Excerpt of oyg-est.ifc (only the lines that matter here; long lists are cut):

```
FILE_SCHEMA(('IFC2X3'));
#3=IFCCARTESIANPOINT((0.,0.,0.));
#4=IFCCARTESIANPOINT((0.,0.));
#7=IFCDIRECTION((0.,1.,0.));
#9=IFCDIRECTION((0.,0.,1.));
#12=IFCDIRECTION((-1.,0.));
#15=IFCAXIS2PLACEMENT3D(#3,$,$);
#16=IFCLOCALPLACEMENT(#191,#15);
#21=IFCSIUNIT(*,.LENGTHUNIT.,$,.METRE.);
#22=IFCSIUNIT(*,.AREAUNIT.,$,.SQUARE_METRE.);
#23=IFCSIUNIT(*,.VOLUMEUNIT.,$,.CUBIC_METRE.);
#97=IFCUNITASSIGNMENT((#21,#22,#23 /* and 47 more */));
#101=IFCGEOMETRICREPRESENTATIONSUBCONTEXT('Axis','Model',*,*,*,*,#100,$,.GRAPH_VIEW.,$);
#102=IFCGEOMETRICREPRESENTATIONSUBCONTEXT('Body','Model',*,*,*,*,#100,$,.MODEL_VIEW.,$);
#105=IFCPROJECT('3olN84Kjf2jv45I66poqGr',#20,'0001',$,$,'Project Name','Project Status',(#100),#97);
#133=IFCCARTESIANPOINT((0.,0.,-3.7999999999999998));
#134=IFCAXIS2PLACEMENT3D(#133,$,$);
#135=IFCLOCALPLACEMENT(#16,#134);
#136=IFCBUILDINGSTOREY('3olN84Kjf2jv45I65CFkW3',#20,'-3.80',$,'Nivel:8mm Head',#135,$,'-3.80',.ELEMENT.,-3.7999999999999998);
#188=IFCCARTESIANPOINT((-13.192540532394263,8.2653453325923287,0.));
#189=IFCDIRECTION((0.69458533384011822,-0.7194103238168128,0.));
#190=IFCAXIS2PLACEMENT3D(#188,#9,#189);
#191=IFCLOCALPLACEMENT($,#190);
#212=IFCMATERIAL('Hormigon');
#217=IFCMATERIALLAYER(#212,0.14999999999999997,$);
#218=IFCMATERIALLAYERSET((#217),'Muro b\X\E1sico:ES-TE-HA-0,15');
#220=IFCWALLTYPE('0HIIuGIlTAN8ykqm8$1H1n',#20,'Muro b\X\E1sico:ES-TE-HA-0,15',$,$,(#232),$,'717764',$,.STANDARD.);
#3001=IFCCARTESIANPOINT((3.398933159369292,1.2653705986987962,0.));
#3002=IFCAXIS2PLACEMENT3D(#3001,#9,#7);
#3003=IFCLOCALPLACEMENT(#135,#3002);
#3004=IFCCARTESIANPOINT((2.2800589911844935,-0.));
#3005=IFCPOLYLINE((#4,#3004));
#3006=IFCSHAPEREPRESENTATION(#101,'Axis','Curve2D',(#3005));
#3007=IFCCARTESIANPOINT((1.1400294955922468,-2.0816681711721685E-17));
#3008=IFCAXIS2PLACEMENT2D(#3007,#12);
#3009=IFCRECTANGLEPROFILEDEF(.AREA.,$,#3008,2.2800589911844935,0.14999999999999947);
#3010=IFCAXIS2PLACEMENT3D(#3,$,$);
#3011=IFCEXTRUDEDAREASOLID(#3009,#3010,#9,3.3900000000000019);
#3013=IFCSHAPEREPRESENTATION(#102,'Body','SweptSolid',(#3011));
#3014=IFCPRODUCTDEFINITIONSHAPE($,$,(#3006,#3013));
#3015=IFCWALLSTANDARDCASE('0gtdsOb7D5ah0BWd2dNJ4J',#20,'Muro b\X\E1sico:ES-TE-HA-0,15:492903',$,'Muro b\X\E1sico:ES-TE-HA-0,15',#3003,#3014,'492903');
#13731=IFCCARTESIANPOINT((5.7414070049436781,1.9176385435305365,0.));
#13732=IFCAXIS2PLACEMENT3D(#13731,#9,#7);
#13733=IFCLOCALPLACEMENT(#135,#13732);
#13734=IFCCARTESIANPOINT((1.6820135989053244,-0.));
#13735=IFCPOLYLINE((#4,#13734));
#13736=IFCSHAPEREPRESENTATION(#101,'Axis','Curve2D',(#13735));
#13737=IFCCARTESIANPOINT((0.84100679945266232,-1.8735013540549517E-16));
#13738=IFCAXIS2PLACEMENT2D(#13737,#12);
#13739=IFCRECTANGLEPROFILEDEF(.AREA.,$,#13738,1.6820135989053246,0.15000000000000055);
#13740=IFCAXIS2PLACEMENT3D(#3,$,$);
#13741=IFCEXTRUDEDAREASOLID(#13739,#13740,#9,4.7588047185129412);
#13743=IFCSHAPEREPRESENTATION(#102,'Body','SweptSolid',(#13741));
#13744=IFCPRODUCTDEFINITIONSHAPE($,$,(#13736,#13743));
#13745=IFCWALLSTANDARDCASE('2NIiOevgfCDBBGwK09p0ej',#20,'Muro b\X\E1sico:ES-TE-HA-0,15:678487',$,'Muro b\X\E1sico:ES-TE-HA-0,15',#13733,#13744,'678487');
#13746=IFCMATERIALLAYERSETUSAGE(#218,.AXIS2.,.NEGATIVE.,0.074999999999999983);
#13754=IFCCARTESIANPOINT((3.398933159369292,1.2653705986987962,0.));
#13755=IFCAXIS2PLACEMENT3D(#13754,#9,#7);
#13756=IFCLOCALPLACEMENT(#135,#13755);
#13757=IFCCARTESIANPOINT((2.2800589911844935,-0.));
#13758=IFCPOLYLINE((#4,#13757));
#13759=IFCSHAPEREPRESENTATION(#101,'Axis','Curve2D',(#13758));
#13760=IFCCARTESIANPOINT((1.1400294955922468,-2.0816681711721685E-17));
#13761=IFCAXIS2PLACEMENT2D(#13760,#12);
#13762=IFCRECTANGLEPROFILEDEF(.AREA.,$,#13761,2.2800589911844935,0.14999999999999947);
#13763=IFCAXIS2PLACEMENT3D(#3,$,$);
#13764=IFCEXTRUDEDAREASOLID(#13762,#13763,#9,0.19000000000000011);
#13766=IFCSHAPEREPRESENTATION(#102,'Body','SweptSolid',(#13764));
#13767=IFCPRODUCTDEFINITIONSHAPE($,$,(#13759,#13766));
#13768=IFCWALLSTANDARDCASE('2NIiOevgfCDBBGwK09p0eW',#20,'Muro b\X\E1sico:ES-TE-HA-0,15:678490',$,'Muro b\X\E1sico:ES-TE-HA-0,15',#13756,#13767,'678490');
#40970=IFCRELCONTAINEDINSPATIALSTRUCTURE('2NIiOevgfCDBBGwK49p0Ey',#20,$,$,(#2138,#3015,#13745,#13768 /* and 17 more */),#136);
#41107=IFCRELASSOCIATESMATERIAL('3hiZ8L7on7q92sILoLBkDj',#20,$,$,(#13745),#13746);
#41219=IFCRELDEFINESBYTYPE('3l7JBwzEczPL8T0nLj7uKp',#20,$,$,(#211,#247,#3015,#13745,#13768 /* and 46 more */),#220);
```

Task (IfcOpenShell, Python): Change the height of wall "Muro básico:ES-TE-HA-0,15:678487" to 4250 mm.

```python
import ifcopenshell
import ifcopenshell.geom
import ifcopenshell.util.representation
import ifcopenshell.util.shape
import ifcopenshell.util.unit

model = ifcopenshell.open("oyg-est.ifc")
unit_scale = ifcopenshell.util.unit.calculate_unit_scale(model)
settings = ifcopenshell.geom.settings()


def volume(element):
    """Net volume in cubic metres, openings subtracted."""
    shape = ifcopenshell.geom.create_shape(settings, element)
    return ifcopenshell.util.shape.get_volume(shape.geometry)


wall = model.by_guid("2NIiOevgfCDBBGwK09p0ej")
before = volume(wall)

body = ifcopenshell.util.representation.get_representation(wall, "Model", "Body")
solid = body.Items[0]
old_height = solid.Depth
solid.Depth = 4.25 / unit_scale
after = volume(wall)

print(f"height {old_height:g} -> {solid.Depth:g}, volume {before:.3f} -> {after:.3f} m3")

model.write("oyg-est_edited.ifc")
```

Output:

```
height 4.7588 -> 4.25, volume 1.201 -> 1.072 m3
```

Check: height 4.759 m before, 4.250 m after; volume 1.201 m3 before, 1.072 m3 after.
